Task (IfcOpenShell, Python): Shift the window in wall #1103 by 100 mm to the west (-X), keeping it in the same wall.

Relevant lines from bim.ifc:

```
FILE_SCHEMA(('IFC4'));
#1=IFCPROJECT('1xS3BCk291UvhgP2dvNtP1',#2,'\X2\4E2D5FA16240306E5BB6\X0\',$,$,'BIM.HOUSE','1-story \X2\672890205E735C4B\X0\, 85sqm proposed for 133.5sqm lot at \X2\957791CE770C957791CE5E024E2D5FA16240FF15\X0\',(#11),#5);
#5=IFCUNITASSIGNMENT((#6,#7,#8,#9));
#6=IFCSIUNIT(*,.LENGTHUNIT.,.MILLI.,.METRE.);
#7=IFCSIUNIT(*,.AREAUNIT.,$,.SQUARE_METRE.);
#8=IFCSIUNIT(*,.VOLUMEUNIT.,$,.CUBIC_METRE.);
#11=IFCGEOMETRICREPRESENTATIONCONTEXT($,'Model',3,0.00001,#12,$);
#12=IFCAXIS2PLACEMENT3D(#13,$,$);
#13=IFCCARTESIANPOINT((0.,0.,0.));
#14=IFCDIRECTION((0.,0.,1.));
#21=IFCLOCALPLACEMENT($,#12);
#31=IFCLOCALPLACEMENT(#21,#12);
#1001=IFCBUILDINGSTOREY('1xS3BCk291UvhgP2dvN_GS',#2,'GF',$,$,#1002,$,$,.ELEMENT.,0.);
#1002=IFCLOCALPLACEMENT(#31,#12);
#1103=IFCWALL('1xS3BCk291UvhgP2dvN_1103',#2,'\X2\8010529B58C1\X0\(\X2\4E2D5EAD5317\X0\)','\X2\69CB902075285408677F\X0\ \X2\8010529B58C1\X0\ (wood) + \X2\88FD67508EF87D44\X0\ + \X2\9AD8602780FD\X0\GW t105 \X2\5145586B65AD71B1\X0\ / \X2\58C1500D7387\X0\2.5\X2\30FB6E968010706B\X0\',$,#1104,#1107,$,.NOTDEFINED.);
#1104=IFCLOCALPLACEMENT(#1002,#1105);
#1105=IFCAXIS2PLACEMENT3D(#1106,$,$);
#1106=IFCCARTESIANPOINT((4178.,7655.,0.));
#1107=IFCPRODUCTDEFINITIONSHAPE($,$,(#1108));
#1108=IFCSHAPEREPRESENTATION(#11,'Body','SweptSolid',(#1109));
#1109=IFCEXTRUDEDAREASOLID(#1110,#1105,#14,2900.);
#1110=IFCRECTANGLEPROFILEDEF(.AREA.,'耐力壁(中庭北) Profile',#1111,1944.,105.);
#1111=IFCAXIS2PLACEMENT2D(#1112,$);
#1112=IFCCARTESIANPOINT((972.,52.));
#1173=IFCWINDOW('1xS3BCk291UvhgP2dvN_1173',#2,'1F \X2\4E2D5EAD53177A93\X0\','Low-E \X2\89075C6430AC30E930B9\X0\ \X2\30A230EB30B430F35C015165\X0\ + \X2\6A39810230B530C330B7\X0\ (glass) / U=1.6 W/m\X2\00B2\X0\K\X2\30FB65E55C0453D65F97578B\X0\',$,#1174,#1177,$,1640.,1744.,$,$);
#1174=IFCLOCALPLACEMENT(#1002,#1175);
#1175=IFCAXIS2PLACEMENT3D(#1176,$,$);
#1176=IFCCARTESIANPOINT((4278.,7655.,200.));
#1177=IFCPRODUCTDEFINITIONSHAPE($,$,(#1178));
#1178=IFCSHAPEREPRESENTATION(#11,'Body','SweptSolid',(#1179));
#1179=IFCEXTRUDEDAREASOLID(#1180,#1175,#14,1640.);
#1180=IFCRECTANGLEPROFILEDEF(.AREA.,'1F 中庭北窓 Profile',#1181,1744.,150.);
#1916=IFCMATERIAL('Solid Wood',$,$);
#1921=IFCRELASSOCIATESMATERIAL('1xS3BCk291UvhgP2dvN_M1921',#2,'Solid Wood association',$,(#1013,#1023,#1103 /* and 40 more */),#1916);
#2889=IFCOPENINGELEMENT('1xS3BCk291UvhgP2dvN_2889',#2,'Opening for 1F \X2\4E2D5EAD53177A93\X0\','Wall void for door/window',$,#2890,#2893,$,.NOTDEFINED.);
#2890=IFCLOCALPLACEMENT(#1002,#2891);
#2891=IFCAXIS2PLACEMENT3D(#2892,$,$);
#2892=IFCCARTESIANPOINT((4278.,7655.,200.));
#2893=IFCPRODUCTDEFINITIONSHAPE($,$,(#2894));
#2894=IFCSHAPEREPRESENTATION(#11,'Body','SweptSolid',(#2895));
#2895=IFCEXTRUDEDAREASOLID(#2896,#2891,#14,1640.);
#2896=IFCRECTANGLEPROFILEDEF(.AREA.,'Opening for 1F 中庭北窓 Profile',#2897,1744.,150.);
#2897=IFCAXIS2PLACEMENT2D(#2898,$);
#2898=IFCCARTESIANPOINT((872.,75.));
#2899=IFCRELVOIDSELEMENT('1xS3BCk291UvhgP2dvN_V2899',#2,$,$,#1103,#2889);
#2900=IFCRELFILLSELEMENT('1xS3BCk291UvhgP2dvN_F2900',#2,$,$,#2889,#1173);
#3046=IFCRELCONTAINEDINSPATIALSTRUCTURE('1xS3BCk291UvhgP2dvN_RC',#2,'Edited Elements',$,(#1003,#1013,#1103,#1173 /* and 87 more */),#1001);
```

```python
import ifcopenshell
import ifcopenshell.api.geometry
import ifcopenshell.util.placement

model = ifcopenshell.open("bim.ifc")

window = model.by_guid("1xS3BCk291UvhgP2dvN_1173")
opening = window.FillsVoids[0].RelatingOpeningElement
wall = opening.VoidsElements[0].RelatingBuildingElement

wall_matrix = ifcopenshell.util.placement.get_local_placement(wall.ObjectPlacement)
shift = wall_matrix[:3, 0] * -100.0
before = ifcopenshell.util.placement.get_local_placement(window.ObjectPlacement)[:3, 3].copy()

# The window is not placed relative to its opening, so move both.
for product in (opening, window):
    matrix = ifcopenshell.util.placement.get_local_placement(product.ObjectPlacement)
    matrix[:3, 3] += shift
    ifcopenshell.api.geometry.edit_object_placement(model, product=product, matrix=matrix, is_si=False)

after = ifcopenshell.util.placement.get_local_placement(window.ObjectPlacement)[:3, 3]
print("window moved by", (after - before).round(3) + 0.0)

model.write("bim_v2.ifc")
```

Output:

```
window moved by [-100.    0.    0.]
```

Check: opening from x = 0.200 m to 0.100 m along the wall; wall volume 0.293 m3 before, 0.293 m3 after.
